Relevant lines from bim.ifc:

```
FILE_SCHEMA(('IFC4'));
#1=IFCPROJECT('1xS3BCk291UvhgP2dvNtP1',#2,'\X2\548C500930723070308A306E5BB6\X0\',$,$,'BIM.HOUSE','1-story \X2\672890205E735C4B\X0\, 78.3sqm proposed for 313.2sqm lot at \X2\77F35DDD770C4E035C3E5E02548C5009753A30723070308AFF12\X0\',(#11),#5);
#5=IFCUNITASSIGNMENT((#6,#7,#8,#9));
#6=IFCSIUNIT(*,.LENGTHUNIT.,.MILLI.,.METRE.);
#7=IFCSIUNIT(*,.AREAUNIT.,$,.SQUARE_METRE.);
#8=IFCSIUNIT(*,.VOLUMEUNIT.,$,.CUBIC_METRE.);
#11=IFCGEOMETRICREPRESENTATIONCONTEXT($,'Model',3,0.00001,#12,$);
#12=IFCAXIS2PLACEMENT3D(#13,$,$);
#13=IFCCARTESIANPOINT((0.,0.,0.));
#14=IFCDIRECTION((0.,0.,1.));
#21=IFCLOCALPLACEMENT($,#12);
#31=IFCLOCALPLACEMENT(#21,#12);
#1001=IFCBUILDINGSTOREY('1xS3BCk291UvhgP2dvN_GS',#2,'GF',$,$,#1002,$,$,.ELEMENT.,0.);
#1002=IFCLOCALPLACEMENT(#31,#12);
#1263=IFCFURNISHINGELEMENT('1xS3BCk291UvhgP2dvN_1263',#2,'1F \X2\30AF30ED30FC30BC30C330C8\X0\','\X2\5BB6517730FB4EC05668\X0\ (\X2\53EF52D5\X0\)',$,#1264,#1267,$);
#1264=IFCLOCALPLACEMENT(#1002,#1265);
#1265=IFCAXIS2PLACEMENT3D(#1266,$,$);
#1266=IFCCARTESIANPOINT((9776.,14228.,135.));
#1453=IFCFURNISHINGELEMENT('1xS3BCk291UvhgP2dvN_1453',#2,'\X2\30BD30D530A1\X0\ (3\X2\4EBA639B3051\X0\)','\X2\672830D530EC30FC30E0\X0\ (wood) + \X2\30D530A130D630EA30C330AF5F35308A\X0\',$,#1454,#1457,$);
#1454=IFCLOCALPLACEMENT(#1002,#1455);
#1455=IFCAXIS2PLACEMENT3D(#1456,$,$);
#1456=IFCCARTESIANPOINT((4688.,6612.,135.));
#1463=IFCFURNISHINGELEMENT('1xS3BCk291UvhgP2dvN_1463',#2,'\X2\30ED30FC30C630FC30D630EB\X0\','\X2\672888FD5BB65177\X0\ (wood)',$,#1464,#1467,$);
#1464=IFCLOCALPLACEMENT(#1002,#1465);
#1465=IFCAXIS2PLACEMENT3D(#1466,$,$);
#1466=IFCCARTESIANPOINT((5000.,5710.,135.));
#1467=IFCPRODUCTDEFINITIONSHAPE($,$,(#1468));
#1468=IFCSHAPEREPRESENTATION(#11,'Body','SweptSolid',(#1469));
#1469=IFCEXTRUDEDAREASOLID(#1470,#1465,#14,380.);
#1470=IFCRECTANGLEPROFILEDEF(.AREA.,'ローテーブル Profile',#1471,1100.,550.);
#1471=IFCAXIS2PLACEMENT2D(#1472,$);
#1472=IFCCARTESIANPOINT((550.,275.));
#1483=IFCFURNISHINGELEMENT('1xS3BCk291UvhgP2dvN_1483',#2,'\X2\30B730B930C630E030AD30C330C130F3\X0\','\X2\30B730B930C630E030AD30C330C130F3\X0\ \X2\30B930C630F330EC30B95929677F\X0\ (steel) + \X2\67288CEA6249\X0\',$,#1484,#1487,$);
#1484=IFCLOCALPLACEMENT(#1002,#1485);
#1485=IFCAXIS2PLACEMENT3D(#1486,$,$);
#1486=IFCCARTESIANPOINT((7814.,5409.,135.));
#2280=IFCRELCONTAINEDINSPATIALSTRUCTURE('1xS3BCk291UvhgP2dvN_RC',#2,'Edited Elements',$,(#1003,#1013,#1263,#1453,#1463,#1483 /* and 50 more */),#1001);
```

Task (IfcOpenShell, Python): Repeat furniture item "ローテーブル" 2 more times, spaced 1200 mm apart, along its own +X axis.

```python
import ifcopenshell
import ifcopenshell.api.geometry
import ifcopenshell.api.root
import ifcopenshell.util.element
import ifcopenshell.util.placement

model = ifcopenshell.open("bim.ifc")


def reuse_history(source, copy):
    """copy_class also copies each property set's owner history, people and application; keep the originals."""
    for rel in copy.IsDefinedBy:
        if rel.is_a("IfcRelDefinesByProperties") and (history := rel.RelatingPropertyDefinition.OwnerHistory):
            rel.RelatingPropertyDefinition.OwnerHistory = source.OwnerHistory
            ifcopenshell.util.element.remove_deep2(model, history)


source = model.by_guid("1xS3BCk291UvhgP2dvN_1463")
base = ifcopenshell.util.placement.get_local_placement(source.ObjectPlacement)
step = base[:3, 0] * 1200.0

for i in range(1, 3):
    copy = ifcopenshell.api.root.copy_class(model, product=source)
    copy.Representation = ifcopenshell.util.element.copy_deep(
        model, source.Representation, exclude=["IfcGeometricRepresentationContext", "IfcRepresentationMap"]
    )
    reuse_history(source, copy)
    matrix = base.copy()
    matrix[:3, 3] += i * step
    print("added at", matrix[:3, 3].round(3) + 0.0)
    ifcopenshell.api.geometry.edit_object_placement(model, product=copy, matrix=matrix, is_si=False)

model.write("bim_rev.ifc")
```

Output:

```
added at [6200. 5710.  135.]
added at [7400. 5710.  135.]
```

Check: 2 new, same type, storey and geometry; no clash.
